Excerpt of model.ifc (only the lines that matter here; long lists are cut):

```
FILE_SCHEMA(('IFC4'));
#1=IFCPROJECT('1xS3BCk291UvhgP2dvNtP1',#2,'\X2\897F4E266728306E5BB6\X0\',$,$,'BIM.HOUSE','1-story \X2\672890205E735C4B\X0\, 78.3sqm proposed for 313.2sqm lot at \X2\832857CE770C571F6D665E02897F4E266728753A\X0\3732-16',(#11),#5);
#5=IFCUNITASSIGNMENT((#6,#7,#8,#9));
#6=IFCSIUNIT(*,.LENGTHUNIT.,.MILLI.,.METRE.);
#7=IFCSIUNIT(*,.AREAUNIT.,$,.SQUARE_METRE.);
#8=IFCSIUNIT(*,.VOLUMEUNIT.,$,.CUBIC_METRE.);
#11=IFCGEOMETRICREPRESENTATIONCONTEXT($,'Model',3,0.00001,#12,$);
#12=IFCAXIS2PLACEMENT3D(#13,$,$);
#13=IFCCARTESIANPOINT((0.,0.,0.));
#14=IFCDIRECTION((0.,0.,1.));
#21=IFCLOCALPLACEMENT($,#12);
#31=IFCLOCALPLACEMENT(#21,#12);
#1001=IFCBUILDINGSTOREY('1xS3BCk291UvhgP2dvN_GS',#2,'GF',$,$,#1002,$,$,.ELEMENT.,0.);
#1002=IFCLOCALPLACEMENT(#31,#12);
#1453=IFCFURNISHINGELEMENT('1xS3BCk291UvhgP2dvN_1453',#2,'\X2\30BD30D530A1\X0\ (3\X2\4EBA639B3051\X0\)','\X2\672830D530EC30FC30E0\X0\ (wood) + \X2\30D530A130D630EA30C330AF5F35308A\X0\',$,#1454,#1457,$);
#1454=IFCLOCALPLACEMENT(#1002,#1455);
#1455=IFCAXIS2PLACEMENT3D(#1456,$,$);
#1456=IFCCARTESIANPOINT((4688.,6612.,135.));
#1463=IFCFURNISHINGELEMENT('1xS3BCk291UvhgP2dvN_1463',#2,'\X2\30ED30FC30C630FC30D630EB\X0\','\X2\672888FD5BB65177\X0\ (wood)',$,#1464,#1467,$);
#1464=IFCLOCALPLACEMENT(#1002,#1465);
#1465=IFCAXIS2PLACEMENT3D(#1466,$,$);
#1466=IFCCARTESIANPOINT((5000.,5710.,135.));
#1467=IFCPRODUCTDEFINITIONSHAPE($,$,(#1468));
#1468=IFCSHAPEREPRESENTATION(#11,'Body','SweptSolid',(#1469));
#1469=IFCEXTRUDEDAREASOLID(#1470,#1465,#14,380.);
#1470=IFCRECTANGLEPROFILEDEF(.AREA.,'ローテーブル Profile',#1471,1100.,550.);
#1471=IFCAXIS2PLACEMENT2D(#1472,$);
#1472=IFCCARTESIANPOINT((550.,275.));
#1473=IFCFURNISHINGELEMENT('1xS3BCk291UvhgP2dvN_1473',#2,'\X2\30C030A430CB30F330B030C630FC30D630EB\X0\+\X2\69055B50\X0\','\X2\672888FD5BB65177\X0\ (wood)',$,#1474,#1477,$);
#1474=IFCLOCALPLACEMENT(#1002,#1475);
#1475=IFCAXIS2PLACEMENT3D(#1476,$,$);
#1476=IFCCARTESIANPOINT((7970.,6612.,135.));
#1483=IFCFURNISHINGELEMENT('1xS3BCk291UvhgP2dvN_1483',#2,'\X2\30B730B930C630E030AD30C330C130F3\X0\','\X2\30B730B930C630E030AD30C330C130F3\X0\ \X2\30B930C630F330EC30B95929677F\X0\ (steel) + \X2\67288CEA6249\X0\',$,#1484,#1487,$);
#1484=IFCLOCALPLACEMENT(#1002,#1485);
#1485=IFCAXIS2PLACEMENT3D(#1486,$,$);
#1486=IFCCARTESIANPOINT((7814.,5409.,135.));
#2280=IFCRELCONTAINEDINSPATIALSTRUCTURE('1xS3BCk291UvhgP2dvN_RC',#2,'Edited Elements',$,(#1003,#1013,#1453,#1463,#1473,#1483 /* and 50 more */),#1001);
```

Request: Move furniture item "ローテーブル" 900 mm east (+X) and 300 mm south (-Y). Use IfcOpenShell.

```python
import ifcopenshell
import ifcopenshell.api.geometry
import ifcopenshell.util.placement
import ifcopenshell.util.unit

model = ifcopenshell.open("model.ifc")
unit_scale = ifcopenshell.util.unit.calculate_unit_scale(model)

item = model.by_guid("1xS3BCk291UvhgP2dvN_1463")
matrix = ifcopenshell.util.placement.get_local_placement(item.ObjectPlacement)
matrix[0, 3] += 0.9 / unit_scale
matrix[1, 3] -= 0.3 / unit_scale
ifcopenshell.api.geometry.edit_object_placement(model, product=item, matrix=matrix, is_si=False)

print(ifcopenshell.util.placement.get_local_placement(item.ObjectPlacement).round(3) + 0.0)

model.write("model_edited.ifc")
```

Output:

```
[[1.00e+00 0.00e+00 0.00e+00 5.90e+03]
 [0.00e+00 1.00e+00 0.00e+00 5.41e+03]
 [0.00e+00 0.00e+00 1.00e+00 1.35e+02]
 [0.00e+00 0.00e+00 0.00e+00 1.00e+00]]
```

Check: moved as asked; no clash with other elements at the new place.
